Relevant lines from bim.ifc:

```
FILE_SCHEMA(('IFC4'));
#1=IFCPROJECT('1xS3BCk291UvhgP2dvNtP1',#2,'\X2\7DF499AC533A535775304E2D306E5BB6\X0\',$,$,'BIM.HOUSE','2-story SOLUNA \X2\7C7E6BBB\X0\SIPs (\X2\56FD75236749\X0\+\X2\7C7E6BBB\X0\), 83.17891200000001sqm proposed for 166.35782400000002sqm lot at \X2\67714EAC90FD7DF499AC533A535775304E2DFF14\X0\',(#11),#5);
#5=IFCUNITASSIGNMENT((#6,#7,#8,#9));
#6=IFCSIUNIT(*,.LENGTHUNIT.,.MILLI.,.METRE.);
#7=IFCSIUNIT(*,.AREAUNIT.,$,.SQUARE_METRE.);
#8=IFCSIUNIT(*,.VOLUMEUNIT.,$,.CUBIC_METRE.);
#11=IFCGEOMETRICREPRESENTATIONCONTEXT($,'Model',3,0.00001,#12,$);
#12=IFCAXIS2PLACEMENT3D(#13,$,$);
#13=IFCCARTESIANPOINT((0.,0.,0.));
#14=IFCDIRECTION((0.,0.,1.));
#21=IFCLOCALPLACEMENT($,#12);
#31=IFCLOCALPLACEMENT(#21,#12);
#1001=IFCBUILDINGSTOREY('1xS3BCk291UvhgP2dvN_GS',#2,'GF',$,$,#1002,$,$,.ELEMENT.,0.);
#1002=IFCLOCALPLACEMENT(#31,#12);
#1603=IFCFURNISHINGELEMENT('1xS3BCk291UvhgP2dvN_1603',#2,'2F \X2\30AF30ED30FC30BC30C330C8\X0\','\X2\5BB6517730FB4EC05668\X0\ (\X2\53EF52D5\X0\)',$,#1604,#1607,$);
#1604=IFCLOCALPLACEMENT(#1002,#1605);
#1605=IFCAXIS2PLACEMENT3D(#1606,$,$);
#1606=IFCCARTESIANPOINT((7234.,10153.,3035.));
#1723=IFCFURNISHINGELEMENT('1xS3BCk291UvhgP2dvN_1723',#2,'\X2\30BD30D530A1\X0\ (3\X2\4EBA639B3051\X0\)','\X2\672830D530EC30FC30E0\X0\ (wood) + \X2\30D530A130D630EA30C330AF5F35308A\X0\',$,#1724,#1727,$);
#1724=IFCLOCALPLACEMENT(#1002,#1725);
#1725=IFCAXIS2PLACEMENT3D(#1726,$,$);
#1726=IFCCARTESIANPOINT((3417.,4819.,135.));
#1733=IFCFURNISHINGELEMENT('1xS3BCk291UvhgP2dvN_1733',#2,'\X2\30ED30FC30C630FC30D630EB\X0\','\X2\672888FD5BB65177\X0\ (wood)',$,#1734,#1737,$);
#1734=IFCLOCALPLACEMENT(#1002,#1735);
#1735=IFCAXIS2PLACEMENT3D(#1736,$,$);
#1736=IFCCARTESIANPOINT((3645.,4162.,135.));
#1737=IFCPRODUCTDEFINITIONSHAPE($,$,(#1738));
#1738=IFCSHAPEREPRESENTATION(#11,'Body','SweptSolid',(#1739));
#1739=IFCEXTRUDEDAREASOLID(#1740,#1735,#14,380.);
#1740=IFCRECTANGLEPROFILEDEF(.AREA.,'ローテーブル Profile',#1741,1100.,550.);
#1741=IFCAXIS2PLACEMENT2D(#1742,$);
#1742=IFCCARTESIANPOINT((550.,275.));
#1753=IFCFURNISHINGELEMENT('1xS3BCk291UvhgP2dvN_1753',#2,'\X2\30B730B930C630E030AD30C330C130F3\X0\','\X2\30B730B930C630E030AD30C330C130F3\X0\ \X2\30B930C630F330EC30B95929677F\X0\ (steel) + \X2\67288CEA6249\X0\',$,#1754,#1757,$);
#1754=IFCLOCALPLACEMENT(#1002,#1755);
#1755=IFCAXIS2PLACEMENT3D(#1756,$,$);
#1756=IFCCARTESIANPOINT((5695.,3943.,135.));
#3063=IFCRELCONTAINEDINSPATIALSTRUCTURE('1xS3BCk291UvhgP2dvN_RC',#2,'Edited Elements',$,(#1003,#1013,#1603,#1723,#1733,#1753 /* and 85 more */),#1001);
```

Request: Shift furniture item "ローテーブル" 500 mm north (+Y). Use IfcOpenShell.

```python
import ifcopenshell
import ifcopenshell.api.geometry
import ifcopenshell.util.placement
import ifcopenshell.util.unit

model = ifcopenshell.open("bim.ifc")
unit_scale = ifcopenshell.util.unit.calculate_unit_scale(model)

item = model.by_guid("1xS3BCk291UvhgP2dvN_1733")
matrix = ifcopenshell.util.placement.get_local_placement(item.ObjectPlacement)
matrix[1, 3] += 0.5 / unit_scale
ifcopenshell.api.geometry.edit_object_placement(model, product=item, matrix=matrix, is_si=False)

print(ifcopenshell.util.placement.get_local_placement(item.ObjectPlacement).round(3) + 0.0)

model.write("bim_rev.ifc")
```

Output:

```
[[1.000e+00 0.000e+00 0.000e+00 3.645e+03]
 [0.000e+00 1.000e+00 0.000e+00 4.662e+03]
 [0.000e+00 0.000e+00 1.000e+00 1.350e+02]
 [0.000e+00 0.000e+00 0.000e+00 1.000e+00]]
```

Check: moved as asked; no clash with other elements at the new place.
